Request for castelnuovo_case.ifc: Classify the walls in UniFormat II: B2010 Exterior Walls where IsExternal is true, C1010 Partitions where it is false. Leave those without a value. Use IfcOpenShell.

First a look at what the model holds.

```python
import ifcopenshell
import ifcopenshell.util.element

model = ifcopenshell.open("castelnuovo_case.ifc")
print(model.schema)
print("classifications:", [c.Name for c in model.by_type("IfcClassification")])
values = [ifcopenshell.util.element.get_pset(e, "Pset_WallCommon", "IsExternal") for e in model.by_type("IfcWall")]
for value in (True, False, None):
    print("IsExternal", value, values.count(value))
```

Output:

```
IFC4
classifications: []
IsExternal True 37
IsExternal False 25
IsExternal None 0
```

```python
import ifcopenshell
import ifcopenshell.api.classification
import ifcopenshell.util.element

model = ifcopenshell.open("castelnuovo_case.ifc")

system = ifcopenshell.api.classification.add_classification(model, classification="UniFormat II")

walls = model.by_type("IfcWall")
external = {e: ifcopenshell.util.element.get_pset(e, "Pset_WallCommon", "IsExternal") for e in walls}
for flag, code, name in ((True, "B2010", "Exterior Walls"), (False, "C1010", "Partitions")):
    products = [e for e in walls if external[e] is flag]
    ifcopenshell.api.classification.add_reference(
        model, products=products, classification=system, identification=code, name=name
    )
    print(code, len(products))

model.write("castelnuovo_case_rev.ifc")
```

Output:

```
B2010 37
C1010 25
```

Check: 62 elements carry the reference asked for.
